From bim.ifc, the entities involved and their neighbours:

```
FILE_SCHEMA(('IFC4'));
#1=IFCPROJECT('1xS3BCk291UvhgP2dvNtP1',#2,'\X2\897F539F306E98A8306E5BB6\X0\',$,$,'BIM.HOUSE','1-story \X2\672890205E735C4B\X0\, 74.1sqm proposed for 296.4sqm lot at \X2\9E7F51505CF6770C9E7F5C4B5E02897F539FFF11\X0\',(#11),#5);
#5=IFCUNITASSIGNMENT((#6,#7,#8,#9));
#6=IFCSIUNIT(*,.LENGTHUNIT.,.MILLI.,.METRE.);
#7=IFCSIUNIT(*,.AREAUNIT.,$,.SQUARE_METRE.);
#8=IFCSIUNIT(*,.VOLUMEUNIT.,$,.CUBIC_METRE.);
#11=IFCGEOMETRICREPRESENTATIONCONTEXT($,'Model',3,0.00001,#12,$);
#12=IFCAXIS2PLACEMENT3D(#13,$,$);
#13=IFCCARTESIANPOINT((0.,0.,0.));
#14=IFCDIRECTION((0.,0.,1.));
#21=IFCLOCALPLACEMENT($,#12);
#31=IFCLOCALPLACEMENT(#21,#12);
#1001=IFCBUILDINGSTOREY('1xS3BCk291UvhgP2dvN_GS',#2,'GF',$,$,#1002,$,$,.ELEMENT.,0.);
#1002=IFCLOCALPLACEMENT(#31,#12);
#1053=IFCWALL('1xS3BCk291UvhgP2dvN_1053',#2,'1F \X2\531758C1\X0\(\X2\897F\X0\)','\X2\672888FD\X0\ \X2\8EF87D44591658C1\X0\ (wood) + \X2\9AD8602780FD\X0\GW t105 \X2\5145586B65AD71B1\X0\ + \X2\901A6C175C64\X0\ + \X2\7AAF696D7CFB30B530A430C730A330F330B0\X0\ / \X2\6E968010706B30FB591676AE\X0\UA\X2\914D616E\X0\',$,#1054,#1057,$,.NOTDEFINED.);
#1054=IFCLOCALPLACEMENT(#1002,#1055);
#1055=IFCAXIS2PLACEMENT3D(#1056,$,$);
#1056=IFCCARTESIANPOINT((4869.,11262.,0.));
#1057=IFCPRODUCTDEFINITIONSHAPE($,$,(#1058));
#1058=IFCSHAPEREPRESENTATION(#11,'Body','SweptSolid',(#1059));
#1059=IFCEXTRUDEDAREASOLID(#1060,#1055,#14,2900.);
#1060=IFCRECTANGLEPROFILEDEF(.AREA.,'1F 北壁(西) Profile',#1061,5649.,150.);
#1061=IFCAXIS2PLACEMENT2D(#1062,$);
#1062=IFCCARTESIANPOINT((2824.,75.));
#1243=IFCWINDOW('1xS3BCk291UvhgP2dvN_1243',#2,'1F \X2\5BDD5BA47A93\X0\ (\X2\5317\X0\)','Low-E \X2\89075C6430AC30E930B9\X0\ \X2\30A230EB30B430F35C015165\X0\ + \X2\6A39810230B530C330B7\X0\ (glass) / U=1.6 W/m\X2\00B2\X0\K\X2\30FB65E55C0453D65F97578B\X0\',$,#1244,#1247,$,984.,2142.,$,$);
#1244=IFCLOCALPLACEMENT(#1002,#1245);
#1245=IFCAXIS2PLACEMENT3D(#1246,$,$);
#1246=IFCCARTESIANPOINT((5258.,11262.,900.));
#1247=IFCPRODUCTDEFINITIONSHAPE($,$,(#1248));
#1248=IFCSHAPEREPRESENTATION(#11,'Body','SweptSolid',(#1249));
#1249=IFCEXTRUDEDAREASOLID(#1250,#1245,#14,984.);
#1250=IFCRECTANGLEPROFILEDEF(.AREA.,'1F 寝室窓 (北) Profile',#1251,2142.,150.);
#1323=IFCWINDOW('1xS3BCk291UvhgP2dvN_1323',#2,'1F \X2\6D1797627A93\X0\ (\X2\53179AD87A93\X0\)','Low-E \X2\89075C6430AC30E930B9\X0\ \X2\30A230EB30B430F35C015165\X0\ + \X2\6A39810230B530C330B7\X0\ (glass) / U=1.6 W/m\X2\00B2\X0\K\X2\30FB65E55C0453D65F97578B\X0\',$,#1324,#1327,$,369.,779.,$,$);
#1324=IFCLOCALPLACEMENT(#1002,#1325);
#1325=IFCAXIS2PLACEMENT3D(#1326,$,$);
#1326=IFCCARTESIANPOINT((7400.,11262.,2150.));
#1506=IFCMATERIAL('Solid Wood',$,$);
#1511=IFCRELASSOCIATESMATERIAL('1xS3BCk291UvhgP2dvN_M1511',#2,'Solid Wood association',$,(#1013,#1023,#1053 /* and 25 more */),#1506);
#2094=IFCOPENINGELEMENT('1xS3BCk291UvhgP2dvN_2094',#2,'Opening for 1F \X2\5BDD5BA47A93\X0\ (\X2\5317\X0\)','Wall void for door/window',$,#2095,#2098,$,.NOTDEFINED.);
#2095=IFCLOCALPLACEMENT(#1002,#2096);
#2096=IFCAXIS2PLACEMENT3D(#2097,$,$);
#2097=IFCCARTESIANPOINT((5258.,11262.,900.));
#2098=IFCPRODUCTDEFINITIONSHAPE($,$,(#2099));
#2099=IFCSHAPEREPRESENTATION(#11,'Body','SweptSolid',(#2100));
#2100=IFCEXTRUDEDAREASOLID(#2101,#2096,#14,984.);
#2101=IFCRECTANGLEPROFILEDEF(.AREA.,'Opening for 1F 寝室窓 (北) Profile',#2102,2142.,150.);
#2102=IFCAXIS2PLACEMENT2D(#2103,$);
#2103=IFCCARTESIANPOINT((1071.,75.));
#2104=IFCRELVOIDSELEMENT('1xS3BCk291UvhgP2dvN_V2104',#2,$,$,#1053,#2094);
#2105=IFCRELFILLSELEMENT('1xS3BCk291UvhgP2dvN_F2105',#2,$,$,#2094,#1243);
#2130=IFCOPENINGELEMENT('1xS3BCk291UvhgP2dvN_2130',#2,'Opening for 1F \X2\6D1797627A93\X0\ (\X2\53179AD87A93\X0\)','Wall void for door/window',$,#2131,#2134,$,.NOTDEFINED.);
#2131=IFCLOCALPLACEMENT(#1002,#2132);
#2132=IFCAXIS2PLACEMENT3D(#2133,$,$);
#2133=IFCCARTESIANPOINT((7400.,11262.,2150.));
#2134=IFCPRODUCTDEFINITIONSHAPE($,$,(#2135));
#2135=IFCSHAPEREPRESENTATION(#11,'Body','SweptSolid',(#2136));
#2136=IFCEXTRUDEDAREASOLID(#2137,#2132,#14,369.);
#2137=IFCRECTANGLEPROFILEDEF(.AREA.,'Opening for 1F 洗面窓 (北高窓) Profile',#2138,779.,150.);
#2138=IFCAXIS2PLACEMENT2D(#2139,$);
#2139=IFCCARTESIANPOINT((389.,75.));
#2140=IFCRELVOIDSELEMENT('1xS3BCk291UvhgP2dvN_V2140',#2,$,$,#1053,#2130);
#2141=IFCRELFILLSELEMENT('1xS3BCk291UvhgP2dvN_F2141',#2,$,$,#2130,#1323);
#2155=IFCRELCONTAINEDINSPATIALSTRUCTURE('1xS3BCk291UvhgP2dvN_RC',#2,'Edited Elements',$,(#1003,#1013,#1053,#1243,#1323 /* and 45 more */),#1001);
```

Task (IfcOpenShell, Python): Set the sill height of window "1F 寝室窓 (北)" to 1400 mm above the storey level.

```python
import numpy as np
import ifcopenshell
import ifcopenshell.api.geometry
import ifcopenshell.geom
import ifcopenshell.util.element
import ifcopenshell.util.placement
import ifcopenshell.util.shape
import ifcopenshell.util.unit

model = ifcopenshell.open("bim.ifc")
unit_scale = ifcopenshell.util.unit.calculate_unit_scale(model)

window = model.by_guid("1xS3BCk291UvhgP2dvN_1243")
opening = window.FillsVoids[0].RelatingOpeningElement
storey = ifcopenshell.util.element.get_container(window, ifc_class="IfcBuildingStorey")
level = ifcopenshell.util.placement.get_local_placement(storey.ObjectPlacement)[2, 3]

# The opening's origin need not be at the sill, so measure its lowest point.
shape = ifcopenshell.geom.create_shape(ifcopenshell.geom.settings(), opening)
bottom = ifcopenshell.util.shape.get_shape_bottom_elevation(shape, shape.geometry) / unit_scale
dz = level + 1.4 / unit_scale - bottom

shift = np.array([0.0, 0.0, dz])
# The window is not placed relative to its opening, so move both.
for product in (opening, window):
    matrix = ifcopenshell.util.placement.get_local_placement(product.ObjectPlacement)
    matrix[:3, 3] += shift
    ifcopenshell.api.geometry.edit_object_placement(model, product=product, matrix=matrix, is_si=False)

print(f"moved by {dz * unit_scale:+.3f} m")

model.write("bim_edited.ifc")
```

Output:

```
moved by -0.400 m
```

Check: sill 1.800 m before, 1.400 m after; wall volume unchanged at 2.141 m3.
